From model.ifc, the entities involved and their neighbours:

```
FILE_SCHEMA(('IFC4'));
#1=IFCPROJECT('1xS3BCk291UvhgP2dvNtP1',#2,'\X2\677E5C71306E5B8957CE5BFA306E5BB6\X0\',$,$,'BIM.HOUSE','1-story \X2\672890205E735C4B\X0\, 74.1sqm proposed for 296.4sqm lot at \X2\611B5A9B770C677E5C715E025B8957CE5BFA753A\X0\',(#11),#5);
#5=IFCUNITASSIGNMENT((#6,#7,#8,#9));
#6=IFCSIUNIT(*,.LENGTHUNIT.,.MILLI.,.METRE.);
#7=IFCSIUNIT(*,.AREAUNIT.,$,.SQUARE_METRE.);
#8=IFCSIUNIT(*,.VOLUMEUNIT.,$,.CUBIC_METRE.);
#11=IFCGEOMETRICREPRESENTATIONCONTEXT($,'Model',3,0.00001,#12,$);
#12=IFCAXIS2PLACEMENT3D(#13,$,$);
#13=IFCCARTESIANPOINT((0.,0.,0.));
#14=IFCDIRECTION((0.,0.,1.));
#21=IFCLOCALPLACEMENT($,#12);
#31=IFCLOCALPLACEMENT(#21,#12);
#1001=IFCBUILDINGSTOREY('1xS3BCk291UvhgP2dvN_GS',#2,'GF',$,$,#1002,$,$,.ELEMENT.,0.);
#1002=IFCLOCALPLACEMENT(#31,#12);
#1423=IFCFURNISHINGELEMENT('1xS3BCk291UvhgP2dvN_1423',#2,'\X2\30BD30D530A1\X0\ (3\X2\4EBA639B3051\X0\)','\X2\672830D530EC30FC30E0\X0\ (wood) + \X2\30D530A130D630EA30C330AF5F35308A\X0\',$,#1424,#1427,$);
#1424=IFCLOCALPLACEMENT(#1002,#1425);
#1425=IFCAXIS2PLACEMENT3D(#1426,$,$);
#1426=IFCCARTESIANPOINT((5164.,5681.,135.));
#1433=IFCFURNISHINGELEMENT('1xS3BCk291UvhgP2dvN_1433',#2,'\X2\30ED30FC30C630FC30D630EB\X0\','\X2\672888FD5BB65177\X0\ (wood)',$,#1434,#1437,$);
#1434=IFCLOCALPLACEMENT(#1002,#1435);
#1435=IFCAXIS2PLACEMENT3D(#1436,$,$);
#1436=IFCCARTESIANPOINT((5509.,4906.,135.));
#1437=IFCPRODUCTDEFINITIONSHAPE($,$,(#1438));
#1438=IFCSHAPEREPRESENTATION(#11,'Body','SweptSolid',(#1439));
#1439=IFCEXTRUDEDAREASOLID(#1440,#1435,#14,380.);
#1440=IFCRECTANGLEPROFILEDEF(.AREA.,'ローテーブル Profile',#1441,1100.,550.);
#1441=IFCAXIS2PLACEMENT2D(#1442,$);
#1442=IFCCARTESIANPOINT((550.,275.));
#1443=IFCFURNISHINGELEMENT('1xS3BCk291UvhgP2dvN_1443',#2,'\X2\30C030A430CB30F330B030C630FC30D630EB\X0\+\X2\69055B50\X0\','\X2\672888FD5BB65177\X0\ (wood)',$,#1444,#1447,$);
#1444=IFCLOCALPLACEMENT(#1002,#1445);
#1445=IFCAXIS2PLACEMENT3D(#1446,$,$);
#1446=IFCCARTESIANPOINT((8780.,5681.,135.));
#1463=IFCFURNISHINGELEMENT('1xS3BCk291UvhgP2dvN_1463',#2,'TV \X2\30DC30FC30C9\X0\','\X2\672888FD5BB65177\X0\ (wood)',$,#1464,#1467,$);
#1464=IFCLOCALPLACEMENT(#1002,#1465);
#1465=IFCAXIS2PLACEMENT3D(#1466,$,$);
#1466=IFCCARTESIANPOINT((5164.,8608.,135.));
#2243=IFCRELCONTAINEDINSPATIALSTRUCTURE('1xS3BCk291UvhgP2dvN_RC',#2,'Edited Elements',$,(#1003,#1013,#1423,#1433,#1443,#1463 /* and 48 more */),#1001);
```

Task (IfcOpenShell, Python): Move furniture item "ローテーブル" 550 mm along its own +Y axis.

```python
import ifcopenshell
import ifcopenshell.api.geometry
import ifcopenshell.util.placement

model = ifcopenshell.open("model.ifc")

item = model.by_guid("1xS3BCk291UvhgP2dvN_1433")
matrix = ifcopenshell.util.placement.get_local_placement(item.ObjectPlacement)
matrix[:3, 3] += matrix[:3, 1] * 550.0
ifcopenshell.api.geometry.edit_object_placement(model, product=item, matrix=matrix, is_si=False)

print(ifcopenshell.util.placement.get_local_placement(item.ObjectPlacement).round(3) + 0.0)

model.write("model_edited.ifc")
```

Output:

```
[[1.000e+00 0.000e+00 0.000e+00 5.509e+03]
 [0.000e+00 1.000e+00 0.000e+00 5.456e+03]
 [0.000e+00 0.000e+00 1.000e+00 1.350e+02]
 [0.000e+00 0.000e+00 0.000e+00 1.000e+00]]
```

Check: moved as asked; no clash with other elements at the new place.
